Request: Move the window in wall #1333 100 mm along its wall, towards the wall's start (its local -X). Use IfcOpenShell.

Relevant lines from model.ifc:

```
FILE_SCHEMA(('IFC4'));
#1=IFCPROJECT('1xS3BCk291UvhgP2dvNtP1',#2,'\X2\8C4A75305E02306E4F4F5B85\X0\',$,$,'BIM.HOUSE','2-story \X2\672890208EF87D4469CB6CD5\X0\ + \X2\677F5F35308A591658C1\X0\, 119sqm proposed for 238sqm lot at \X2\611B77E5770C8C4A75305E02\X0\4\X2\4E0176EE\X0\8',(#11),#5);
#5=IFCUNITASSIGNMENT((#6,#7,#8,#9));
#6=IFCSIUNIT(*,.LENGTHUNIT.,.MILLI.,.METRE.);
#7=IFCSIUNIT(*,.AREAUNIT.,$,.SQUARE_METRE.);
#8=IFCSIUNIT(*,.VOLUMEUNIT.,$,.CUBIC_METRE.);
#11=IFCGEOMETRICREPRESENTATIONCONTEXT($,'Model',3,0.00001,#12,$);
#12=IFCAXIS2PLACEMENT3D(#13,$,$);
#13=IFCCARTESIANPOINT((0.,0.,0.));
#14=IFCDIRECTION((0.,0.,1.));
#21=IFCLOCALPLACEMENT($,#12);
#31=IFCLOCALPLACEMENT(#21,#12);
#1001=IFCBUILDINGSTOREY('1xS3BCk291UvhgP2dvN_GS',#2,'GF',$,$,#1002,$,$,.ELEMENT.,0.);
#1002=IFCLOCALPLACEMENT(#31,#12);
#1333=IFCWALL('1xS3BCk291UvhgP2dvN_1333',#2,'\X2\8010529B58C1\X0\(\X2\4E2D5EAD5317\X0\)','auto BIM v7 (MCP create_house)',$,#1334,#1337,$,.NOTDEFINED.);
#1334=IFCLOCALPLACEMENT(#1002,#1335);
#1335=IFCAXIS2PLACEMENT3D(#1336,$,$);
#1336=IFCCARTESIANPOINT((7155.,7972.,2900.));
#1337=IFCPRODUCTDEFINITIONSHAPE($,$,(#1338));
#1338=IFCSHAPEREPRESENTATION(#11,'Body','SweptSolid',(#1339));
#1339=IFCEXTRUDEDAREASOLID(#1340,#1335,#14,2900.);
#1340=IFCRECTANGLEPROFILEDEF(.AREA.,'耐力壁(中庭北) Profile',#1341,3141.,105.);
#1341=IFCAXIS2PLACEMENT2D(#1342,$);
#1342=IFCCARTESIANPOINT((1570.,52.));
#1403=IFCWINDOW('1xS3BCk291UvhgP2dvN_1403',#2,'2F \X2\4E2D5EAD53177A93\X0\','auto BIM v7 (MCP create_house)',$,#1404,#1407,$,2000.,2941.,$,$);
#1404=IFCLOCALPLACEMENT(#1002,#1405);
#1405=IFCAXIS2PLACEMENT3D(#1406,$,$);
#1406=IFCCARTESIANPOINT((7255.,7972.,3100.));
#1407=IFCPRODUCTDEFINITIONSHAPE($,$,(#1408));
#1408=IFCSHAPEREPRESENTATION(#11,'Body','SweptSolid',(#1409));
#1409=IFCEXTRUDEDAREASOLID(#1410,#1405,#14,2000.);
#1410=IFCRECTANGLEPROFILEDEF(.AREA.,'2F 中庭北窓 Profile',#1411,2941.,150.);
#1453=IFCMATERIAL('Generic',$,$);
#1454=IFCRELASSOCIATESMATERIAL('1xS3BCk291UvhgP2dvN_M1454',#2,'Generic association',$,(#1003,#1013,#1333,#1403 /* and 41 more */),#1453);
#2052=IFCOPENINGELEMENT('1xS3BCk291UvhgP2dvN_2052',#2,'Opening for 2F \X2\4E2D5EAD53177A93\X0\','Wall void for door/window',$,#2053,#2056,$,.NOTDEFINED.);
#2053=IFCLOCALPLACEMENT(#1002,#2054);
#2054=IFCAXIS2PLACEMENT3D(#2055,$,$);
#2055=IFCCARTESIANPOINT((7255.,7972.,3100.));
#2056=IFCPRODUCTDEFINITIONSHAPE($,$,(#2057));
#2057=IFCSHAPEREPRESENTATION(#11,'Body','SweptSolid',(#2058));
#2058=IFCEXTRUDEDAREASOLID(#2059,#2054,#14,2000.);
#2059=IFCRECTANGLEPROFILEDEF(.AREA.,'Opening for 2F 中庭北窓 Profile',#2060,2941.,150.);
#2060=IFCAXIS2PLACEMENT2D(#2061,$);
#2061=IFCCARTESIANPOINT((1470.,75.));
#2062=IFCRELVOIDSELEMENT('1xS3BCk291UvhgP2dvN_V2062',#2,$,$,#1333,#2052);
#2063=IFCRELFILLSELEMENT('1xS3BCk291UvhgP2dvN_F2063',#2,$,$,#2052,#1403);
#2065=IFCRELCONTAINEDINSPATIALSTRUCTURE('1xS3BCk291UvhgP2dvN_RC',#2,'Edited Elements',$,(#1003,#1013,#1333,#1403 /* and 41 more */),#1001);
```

```python
import ifcopenshell
import ifcopenshell.api.geometry
import ifcopenshell.util.placement
import ifcopenshell.util.unit

model = ifcopenshell.open("model.ifc")
unit_scale = ifcopenshell.util.unit.calculate_unit_scale(model)

window = model.by_guid("1xS3BCk291UvhgP2dvN_1403")
opening = window.FillsVoids[0].RelatingOpeningElement
wall = opening.VoidsElements[0].RelatingBuildingElement

wall_matrix = ifcopenshell.util.placement.get_local_placement(wall.ObjectPlacement)
shift = wall_matrix[:3, 0] * -0.1 / unit_scale
before = ifcopenshell.util.placement.get_local_placement(window.ObjectPlacement)[:3, 3].copy()

# The window is not placed relative to its opening, so move both.
for product in (opening, window):
    matrix = ifcopenshell.util.placement.get_local_placement(product.ObjectPlacement)
    matrix[:3, 3] += shift
    ifcopenshell.api.geometry.edit_object_placement(model, product=product, matrix=matrix, is_si=False)

after = ifcopenshell.util.placement.get_local_placement(window.ObjectPlacement)[:3, 3]
print("window moved by", (after - before).round(3) + 0.0)

model.write("model_updated.ifc")
```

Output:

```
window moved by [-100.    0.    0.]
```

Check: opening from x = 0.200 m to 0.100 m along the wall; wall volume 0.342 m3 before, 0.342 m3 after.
